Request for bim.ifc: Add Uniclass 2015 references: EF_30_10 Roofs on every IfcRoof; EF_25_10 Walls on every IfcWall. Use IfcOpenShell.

First a look at what the model holds.

```python
import ifcopenshell

model = ifcopenshell.open("bim.ifc")
print(model.schema)
print("classifications:", [c.Name for c in model.by_type("IfcClassification")])
for ifc_class in ("IfcDoor", "IfcRoof", "IfcStair", "IfcWall", "IfcWindow"):
    print(ifc_class, len(model.by_type(ifc_class)))
```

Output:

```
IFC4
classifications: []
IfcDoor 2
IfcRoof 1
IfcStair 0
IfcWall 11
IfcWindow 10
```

```python
import ifcopenshell
import ifcopenshell.api.classification

model = ifcopenshell.open("bim.ifc")

system = ifcopenshell.api.classification.add_classification(model, classification="Uniclass 2015")

codes = {
    "IfcRoof": ("EF_30_10", "Roofs"),
    "IfcWall": ("EF_25_10", "Walls"),
}
for ifc_class, (code, name) in codes.items():
    products = model.by_type(ifc_class)
    ifcopenshell.api.classification.add_reference(
        model, products=products, classification=system, identification=code, name=name
    )
    print(code, len(products))

model.write("bim_edited.ifc")
```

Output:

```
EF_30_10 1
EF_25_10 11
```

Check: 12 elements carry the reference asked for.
